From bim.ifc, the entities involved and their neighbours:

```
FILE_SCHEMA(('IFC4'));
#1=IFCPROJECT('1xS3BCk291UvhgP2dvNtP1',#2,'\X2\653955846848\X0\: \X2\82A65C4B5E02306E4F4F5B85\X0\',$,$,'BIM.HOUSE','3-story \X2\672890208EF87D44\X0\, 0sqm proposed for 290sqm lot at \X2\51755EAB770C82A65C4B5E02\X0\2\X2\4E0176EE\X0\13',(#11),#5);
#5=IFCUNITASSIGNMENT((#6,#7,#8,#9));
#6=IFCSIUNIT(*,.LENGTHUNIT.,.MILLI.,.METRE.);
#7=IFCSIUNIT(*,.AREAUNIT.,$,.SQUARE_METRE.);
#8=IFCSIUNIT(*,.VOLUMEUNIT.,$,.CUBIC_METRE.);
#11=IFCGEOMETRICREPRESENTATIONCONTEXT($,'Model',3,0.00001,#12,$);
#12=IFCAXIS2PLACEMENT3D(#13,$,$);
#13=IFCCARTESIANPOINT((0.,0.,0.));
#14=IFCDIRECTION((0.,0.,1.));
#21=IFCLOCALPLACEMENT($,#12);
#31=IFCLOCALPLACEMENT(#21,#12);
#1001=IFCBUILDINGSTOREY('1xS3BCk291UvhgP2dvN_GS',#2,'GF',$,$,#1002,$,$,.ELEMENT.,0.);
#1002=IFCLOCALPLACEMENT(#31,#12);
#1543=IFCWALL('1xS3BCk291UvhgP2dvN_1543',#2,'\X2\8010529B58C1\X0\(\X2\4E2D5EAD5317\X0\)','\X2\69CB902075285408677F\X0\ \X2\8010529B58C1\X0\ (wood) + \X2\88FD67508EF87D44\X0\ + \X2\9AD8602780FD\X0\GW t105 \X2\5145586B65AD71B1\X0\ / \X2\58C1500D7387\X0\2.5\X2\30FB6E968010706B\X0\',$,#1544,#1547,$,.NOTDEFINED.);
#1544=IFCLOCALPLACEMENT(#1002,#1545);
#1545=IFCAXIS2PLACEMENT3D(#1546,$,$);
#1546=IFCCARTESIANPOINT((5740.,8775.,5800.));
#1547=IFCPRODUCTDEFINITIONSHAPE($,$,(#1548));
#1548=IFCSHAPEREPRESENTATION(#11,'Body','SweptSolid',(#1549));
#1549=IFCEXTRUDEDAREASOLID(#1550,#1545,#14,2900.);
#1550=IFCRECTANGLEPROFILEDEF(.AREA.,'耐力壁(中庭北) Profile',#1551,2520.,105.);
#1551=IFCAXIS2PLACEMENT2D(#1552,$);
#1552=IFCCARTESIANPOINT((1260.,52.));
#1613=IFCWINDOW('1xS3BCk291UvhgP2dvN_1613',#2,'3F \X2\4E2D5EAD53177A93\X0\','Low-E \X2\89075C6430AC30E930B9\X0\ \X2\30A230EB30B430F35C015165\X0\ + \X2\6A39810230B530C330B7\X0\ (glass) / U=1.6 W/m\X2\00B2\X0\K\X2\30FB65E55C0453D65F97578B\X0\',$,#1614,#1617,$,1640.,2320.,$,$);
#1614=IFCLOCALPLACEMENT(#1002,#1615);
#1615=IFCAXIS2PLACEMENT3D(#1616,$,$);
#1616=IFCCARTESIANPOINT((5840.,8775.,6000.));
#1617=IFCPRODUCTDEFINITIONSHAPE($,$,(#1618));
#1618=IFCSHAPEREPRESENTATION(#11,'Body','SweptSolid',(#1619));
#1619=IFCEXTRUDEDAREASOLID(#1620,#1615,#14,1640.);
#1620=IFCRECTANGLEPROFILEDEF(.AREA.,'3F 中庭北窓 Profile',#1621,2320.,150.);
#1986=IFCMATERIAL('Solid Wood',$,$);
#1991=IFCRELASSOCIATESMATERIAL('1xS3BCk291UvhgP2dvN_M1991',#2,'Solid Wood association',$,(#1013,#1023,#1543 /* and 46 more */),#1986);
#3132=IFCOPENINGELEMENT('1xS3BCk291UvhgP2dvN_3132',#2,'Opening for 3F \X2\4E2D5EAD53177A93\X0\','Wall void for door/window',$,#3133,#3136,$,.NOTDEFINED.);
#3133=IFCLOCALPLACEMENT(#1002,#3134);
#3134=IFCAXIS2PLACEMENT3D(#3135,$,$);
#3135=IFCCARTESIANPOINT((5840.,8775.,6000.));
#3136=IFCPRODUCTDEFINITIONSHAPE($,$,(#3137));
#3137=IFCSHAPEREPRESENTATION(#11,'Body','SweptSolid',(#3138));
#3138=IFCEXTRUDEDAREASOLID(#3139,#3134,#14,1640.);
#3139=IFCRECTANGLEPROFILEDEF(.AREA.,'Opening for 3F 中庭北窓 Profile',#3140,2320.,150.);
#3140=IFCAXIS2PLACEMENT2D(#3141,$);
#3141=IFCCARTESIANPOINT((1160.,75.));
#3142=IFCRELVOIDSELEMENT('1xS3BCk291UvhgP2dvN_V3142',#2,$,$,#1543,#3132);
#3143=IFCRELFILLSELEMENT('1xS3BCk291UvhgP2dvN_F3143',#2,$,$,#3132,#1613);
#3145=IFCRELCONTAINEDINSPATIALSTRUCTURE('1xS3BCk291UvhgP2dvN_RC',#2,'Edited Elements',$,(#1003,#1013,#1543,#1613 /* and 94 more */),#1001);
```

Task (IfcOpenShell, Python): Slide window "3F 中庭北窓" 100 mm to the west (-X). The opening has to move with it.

```python
import ifcopenshell
import ifcopenshell.api.geometry
import ifcopenshell.util.placement
import ifcopenshell.util.unit

model = ifcopenshell.open("bim.ifc")
unit_scale = ifcopenshell.util.unit.calculate_unit_scale(model)

window = model.by_id(1613)
opening = window.FillsVoids[0].RelatingOpeningElement
wall = opening.VoidsElements[0].RelatingBuildingElement

wall_matrix = ifcopenshell.util.placement.get_local_placement(wall.ObjectPlacement)
shift = wall_matrix[:3, 0] * -0.1 / unit_scale
before = ifcopenshell.util.placement.get_local_placement(window.ObjectPlacement)[:3, 3].copy()

# The window is not placed relative to its opening, so move both.
for product in (opening, window):
    matrix = ifcopenshell.util.placement.get_local_placement(product.ObjectPlacement)
    matrix[:3, 3] += shift
    ifcopenshell.api.geometry.edit_object_placement(model, product=product, matrix=matrix, is_si=False)

after = ifcopenshell.util.placement.get_local_placement(window.ObjectPlacement)[:3, 3]
print("window moved by", (after - before).round(3) + 0.0)

model.write("bim_edited.ifc")
```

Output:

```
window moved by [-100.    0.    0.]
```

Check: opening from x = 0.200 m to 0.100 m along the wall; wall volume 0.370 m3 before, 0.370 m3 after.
